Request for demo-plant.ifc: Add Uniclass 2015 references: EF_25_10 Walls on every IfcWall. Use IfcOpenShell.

First a look at what the model holds.

```python
import ifcopenshell

model = ifcopenshell.open("demo-plant.ifc")
print(model.schema)
print("classifications:", [c.Name for c in model.by_type("IfcClassification")])
for ifc_class in ("IfcDoor", "IfcRoof", "IfcStair", "IfcWall", "IfcWindow"):
    print(ifc_class, len(model.by_type(ifc_class)))
```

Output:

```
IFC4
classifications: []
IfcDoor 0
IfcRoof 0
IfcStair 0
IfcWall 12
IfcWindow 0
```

```python
import ifcopenshell
import ifcopenshell.api.classification

model = ifcopenshell.open("demo-plant.ifc")

system = ifcopenshell.api.classification.add_classification(model, classification="Uniclass 2015")

codes = {
    "IfcWall": ("EF_25_10", "Walls"),
}
for ifc_class, (code, name) in codes.items():
    products = model.by_type(ifc_class)
    ifcopenshell.api.classification.add_reference(
        model, products=products, classification=system, identification=code, name=name
    )
    print(code, len(products))

model.write("demo-plant_rev.ifc")
```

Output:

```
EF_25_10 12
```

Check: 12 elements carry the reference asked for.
